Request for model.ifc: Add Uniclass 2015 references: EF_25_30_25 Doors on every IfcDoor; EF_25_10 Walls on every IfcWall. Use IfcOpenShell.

First a look at what the model holds.

```python
import ifcopenshell

model = ifcopenshell.open("model.ifc")
print(model.schema)
print("classifications:", [c.Name for c in model.by_type("IfcClassification")])
for ifc_class in ("IfcDoor", "IfcRoof", "IfcStair", "IfcWall", "IfcWindow"):
    print(ifc_class, len(model.by_type(ifc_class)))
```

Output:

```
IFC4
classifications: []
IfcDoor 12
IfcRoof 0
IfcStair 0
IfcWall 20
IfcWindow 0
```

```python
import ifcopenshell
import ifcopenshell.api.classification

model = ifcopenshell.open("model.ifc")

system = ifcopenshell.api.classification.add_classification(model, classification="Uniclass 2015")

codes = {
    "IfcDoor": ("EF_25_30_25", "Doors"),
    "IfcWall": ("EF_25_10", "Walls"),
}
for ifc_class, (code, name) in codes.items():
    products = model.by_type(ifc_class)
    ifcopenshell.api.classification.add_reference(
        model, products=products, classification=system, identification=code, name=name
    )
    print(code, len(products))

model.write("model_updated.ifc")
```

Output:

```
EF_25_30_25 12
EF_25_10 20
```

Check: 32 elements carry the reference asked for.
